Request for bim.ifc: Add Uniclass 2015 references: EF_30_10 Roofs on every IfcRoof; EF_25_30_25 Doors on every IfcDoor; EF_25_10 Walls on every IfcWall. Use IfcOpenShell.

First a look at what the model holds.

```python
import ifcopenshell

model = ifcopenshell.open("bim.ifc")
print(model.schema)
print("classifications:", [c.Name for c in model.by_type("IfcClassification")])
for ifc_class in ("IfcDoor", "IfcRoof", "IfcStair", "IfcWall", "IfcWindow"):
    print(ifc_class, len(model.by_type(ifc_class)))
```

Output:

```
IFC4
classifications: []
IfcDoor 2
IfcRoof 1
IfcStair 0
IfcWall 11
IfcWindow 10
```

```python
import ifcopenshell
import ifcopenshell.api.classification

model = ifcopenshell.open("bim.ifc")

system = ifcopenshell.api.classification.add_classification(model, classification="Uniclass 2015")

codes = {
    "IfcRoof": ("EF_30_10", "Roofs"),
    "IfcDoor": ("EF_25_30_25", "Doors"),
    "IfcWall": ("EF_25_10", "Walls"),
}
for ifc_class, (code, name) in codes.items():
    products = model.by_type(ifc_class)
    ifcopenshell.api.classification.add_reference(
        model, products=products, classification=system, identification=code, name=name
    )
    print(code, len(products))

model.write("bim_updated.ifc")
```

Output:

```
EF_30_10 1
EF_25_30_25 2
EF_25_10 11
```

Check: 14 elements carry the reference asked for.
